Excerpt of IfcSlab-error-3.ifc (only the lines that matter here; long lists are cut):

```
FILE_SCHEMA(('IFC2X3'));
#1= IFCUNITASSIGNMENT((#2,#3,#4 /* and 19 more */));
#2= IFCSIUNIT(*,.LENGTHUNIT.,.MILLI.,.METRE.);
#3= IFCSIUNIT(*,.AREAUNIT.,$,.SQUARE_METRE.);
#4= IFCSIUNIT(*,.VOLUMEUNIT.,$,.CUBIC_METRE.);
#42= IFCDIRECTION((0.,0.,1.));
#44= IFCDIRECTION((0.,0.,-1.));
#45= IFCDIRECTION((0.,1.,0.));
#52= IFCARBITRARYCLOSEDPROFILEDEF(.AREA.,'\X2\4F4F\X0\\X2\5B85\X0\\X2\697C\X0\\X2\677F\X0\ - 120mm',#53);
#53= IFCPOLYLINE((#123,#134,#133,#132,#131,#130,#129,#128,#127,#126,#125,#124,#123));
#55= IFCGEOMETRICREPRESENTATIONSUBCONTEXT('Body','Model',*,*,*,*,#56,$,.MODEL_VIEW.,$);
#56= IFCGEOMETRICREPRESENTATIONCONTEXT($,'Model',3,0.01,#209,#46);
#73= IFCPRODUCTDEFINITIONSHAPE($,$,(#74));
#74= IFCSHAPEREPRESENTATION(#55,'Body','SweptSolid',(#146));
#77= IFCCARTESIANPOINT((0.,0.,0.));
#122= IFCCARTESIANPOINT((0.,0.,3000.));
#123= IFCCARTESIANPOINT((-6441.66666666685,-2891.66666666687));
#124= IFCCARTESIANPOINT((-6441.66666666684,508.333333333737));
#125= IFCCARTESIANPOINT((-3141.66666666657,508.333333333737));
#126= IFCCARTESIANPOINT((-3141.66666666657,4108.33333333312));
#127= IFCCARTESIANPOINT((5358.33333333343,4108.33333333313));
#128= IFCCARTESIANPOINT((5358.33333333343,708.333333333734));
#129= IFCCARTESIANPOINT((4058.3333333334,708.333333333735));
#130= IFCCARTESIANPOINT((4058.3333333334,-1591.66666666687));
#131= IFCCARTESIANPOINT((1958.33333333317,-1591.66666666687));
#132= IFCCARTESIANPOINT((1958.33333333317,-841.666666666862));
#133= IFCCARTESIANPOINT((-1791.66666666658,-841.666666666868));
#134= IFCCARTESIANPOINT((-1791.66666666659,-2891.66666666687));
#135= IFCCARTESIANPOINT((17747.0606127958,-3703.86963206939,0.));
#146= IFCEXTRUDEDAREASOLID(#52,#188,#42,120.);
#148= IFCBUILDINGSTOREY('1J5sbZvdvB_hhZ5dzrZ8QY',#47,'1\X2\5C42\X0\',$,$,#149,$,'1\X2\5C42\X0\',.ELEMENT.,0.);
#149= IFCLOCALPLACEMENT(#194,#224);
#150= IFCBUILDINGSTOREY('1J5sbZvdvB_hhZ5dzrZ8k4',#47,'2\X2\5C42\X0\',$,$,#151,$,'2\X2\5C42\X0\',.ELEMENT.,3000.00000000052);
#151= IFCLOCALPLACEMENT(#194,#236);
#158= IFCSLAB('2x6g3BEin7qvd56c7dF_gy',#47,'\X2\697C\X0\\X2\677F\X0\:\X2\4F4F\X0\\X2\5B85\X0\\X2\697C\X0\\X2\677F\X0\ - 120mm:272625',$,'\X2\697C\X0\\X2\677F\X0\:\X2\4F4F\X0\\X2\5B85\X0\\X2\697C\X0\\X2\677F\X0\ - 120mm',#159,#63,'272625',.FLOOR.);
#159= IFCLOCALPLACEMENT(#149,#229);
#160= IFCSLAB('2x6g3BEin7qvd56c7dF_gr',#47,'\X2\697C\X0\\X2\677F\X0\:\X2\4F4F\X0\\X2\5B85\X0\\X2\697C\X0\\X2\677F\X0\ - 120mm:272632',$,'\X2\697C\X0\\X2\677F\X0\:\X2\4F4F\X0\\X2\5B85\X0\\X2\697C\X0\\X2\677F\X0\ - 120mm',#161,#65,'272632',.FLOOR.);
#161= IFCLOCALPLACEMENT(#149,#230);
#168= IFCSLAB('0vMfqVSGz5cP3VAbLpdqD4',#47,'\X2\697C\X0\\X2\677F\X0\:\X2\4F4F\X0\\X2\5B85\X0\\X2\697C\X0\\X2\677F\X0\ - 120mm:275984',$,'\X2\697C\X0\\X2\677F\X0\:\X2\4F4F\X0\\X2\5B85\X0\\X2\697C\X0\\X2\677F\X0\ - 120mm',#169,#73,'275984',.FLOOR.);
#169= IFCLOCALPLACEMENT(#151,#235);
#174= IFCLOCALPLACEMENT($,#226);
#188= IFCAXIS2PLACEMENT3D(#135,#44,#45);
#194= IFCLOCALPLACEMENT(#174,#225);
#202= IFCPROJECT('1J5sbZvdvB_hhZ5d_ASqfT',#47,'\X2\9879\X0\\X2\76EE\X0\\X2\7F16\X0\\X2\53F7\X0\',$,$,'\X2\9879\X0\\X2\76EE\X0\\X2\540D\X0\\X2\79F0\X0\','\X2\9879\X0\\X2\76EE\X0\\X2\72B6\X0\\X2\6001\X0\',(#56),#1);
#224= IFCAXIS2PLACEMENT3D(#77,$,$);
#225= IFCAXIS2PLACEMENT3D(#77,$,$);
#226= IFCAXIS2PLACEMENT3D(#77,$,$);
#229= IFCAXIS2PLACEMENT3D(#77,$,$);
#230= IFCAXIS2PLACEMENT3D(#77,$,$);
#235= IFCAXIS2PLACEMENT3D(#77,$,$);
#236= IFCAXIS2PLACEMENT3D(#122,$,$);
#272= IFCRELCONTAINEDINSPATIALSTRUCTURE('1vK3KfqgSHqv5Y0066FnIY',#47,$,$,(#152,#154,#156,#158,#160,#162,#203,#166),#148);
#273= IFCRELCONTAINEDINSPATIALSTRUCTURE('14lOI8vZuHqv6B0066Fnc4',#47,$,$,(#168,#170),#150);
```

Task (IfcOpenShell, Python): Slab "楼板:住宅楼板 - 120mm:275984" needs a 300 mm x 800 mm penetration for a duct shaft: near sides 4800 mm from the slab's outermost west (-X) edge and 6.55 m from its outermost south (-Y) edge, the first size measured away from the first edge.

```python
import numpy as np
import ifcopenshell
import ifcopenshell.api.feature
import ifcopenshell.api.geometry
import ifcopenshell.api.root
import ifcopenshell.geom
import ifcopenshell.util.placement
import ifcopenshell.util.representation
import ifcopenshell.util.shape
import ifcopenshell.util.unit

model = ifcopenshell.open("IfcSlab-error-3.ifc")
unit_scale = ifcopenshell.util.unit.calculate_unit_scale(model)
settings = ifcopenshell.geom.settings()


def volume(element):
    """Net volume in cubic metres, openings subtracted."""
    shape = ifcopenshell.geom.create_shape(settings, element)
    return ifcopenshell.util.shape.get_volume(shape.geometry)


slab = model.by_guid("0vMfqVSGz5cP3VAbLpdqD4")
before = volume(slab)

# Extent in the slab's own axes, in metres. The edges named are its -X and -Y sides.
slab_shape = ifcopenshell.geom.create_shape(settings, slab)
vertices = ifcopenshell.util.shape.get_vertices(slab_shape.geometry)
x_min, y_min, bottom = vertices.min(axis=0)
top = vertices[:, 2].max()

opening = ifcopenshell.api.root.create_entity(model, ifc_class="IfcOpeningElement", name="Duct shaft opening")
context = ifcopenshell.util.representation.get_context(model, "Model", "Body", "MODEL_VIEW")
width, depth = 0.3, 0.8
outline = [(0.0, 0.0), (width, 0.0), (width, depth), (0.0, depth), (0.0, 0.0)]
# Overshoot both faces by 50 mm so the cut is clean.
shape = ifcopenshell.api.geometry.add_slab_representation(
    model, context=context, depth=top - bottom + 0.1, polyline=outline
)
ifcopenshell.api.geometry.assign_representation(model, product=opening, representation=shape)

matrix = ifcopenshell.util.placement.get_local_placement(slab.ObjectPlacement)
matrix[:, 3] = matrix @ np.append(np.array([x_min + 4.8, y_min + 6.55, bottom - 0.05]) / unit_scale, 1.0)
ifcopenshell.api.geometry.edit_object_placement(model, product=opening, matrix=matrix, is_si=False)
ifcopenshell.api.feature.add_feature(model, feature=opening, element=slab)

after = volume(slab)

print(f"slab volume {before:.3f} -> {after:.3f} m3")

model.write("IfcSlab-error-3_rev.ifc")
```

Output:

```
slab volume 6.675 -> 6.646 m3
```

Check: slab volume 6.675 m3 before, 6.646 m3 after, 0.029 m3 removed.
